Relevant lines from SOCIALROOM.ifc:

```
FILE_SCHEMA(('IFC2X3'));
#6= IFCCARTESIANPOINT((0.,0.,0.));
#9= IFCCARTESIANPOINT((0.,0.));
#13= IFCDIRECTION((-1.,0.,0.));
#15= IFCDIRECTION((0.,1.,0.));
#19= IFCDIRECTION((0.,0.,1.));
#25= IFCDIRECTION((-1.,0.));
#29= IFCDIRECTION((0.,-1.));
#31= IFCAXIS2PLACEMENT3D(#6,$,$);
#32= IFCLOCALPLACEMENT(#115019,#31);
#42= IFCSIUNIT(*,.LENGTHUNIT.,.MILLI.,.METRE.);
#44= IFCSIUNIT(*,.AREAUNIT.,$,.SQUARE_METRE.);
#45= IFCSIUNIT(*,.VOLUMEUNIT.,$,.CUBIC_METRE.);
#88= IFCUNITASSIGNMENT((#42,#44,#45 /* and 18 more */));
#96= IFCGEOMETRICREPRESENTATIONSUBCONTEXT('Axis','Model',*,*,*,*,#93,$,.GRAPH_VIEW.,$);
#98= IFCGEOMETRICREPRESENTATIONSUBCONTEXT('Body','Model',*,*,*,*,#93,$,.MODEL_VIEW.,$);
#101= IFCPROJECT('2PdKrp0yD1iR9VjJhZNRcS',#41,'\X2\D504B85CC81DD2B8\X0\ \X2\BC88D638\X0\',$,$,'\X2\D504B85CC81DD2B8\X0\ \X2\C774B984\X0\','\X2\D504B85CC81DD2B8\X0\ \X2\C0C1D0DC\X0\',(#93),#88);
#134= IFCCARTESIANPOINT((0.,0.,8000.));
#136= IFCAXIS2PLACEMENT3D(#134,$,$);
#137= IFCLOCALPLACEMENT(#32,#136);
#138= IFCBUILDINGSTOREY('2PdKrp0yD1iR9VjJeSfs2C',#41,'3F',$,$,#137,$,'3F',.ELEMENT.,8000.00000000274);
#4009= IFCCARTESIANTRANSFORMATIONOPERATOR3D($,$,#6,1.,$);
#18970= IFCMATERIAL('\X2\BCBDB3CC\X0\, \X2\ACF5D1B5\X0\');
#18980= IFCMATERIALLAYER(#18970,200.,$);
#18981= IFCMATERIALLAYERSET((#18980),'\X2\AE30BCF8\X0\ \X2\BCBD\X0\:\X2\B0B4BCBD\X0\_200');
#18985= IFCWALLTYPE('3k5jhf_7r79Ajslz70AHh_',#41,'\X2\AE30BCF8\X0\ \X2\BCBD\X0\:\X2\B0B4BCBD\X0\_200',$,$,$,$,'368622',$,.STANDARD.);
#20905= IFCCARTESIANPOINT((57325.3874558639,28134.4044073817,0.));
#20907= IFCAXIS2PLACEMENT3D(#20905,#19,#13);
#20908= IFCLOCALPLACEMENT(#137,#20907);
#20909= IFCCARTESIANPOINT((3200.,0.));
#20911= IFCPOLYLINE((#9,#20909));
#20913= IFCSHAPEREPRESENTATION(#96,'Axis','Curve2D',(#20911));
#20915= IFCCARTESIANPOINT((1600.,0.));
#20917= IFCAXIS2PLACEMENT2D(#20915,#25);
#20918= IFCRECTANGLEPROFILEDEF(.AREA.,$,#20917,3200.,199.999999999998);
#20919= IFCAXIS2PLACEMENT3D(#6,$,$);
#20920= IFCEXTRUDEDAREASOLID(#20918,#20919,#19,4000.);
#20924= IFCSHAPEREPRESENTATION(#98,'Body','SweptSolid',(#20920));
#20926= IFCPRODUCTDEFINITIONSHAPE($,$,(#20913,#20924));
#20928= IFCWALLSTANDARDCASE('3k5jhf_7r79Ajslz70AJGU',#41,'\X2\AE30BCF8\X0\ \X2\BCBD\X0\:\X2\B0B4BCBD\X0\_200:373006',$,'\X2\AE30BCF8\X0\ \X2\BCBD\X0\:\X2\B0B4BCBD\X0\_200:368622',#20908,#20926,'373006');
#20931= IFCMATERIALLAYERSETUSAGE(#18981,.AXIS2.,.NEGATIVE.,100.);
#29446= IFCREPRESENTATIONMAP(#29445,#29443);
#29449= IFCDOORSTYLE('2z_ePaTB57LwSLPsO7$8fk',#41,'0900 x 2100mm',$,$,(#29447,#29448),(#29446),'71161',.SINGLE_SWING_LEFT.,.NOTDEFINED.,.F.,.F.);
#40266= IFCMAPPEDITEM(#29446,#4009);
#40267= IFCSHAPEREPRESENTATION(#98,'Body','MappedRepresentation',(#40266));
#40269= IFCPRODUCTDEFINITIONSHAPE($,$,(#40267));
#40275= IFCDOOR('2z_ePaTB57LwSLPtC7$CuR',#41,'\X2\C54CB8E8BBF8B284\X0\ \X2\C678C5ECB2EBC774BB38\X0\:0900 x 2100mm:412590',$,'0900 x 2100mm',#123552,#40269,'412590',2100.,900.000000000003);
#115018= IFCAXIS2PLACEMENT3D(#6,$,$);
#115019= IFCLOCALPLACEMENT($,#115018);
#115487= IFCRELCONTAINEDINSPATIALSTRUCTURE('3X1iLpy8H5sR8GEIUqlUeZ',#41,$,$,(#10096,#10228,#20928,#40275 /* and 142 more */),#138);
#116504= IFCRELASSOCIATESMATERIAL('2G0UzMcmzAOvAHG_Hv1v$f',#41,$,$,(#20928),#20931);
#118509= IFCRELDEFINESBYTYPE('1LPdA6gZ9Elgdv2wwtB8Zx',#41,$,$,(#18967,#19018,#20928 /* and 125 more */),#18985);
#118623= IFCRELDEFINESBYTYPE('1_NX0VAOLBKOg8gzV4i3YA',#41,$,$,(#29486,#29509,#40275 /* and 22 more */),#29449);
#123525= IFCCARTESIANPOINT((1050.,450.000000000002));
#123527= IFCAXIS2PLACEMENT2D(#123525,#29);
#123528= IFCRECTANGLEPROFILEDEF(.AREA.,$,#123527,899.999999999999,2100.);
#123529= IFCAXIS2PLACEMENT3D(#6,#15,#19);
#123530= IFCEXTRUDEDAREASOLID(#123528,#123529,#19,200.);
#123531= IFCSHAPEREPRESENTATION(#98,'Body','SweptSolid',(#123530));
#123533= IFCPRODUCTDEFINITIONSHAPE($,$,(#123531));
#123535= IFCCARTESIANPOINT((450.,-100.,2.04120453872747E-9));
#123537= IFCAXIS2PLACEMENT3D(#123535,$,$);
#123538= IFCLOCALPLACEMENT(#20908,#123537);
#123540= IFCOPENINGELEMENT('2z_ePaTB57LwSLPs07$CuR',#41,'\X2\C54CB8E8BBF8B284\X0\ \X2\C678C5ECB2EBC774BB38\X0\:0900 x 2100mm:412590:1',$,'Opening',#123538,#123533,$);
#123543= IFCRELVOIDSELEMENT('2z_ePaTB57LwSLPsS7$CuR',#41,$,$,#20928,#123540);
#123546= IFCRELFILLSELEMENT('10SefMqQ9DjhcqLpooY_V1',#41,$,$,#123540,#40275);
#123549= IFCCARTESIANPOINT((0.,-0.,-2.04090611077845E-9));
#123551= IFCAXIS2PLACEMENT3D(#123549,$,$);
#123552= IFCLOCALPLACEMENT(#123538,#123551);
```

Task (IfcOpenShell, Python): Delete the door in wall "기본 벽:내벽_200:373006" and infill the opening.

```python
import ifcopenshell
import ifcopenshell.api.feature
import ifcopenshell.api.root
import ifcopenshell.geom
import ifcopenshell.util.shape

model = ifcopenshell.open("SOCIALROOM.ifc")
settings = ifcopenshell.geom.settings()


def volume(element):
    """Net volume in cubic metres, openings subtracted."""
    shape = ifcopenshell.geom.create_shape(settings, element)
    return ifcopenshell.util.shape.get_volume(shape.geometry)


door = model.by_id(40275)
opening = door.FillsVoids[0].RelatingOpeningElement
wall = opening.VoidsElements[0].RelatingBuildingElement
before = volume(wall)

ifcopenshell.api.root.remove_product(model, product=door)
ifcopenshell.api.feature.remove_feature(model, feature=opening)

after = volume(wall)

print(f"wall volume {before:.3f} -> {after:.3f} m3")

model.write("SOCIALROOM_v2.ifc")
```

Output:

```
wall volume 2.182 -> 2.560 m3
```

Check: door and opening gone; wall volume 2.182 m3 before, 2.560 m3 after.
